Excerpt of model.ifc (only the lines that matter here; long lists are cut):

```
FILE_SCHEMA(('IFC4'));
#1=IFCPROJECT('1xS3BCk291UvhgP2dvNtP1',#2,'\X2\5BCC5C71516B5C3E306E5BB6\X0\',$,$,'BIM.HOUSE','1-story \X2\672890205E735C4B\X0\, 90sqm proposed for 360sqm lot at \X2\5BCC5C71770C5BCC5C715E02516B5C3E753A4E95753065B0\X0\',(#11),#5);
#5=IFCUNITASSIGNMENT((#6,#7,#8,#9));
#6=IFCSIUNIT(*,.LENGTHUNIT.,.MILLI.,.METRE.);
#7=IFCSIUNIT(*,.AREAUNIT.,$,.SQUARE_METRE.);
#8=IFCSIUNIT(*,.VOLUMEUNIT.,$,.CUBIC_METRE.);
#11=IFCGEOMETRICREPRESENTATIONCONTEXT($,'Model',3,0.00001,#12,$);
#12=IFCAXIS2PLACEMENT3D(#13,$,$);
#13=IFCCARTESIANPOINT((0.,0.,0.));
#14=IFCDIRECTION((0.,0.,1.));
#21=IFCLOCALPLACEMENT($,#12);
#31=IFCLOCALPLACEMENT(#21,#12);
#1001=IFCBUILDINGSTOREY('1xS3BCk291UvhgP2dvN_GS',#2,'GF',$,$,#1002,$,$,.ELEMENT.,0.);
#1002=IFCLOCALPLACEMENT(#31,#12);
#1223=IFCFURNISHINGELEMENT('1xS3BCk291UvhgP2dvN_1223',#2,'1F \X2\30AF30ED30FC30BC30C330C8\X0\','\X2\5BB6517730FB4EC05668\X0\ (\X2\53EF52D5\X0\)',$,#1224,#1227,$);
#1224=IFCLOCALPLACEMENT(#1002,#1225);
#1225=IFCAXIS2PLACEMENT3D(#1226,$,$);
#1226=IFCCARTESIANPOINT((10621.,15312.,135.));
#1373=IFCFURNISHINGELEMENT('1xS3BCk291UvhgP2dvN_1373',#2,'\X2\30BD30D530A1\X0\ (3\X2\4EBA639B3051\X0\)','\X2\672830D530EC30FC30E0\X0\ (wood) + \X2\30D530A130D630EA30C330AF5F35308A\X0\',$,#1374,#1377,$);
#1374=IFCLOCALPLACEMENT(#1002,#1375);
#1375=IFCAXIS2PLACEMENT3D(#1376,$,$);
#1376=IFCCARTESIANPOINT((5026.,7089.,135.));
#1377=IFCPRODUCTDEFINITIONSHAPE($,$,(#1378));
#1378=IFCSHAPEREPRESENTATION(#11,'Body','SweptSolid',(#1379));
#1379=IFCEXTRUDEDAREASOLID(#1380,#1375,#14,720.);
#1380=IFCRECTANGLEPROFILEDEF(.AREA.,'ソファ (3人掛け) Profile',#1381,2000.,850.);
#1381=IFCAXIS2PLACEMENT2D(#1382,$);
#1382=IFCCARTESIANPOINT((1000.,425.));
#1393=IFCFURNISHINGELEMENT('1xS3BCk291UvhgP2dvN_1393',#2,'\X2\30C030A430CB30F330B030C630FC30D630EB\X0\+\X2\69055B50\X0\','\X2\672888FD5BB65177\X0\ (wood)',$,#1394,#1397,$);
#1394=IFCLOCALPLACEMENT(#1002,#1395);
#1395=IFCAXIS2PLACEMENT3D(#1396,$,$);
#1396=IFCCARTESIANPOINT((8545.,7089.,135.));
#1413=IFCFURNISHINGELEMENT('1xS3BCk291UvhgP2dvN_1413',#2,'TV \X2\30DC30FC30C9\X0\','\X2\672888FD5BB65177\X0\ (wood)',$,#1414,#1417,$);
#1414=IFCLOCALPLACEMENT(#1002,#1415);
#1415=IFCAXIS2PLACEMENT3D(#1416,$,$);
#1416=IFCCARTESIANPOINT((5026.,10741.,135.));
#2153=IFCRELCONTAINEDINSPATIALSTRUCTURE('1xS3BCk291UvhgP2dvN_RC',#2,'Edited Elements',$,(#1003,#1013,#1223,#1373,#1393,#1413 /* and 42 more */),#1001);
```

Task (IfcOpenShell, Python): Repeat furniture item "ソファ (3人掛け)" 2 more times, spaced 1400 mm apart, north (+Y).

```python
import numpy as np
import ifcopenshell
import ifcopenshell.api.geometry
import ifcopenshell.api.root
import ifcopenshell.util.element
import ifcopenshell.util.placement
import ifcopenshell.util.unit

model = ifcopenshell.open("model.ifc")
unit_scale = ifcopenshell.util.unit.calculate_unit_scale(model)


def reuse_history(source, copy):
    """copy_class also copies each property set's owner history, people and application; keep the originals."""
    for rel in copy.IsDefinedBy:
        if rel.is_a("IfcRelDefinesByProperties") and (history := rel.RelatingPropertyDefinition.OwnerHistory):
            rel.RelatingPropertyDefinition.OwnerHistory = source.OwnerHistory
            ifcopenshell.util.element.remove_deep2(model, history)


source = model.by_guid("1xS3BCk291UvhgP2dvN_1373")
base = ifcopenshell.util.placement.get_local_placement(source.ObjectPlacement)
step = np.array([0.0, 1.0, 0.0]) * 1.4 / unit_scale

for i in range(1, 3):
    copy = ifcopenshell.api.root.copy_class(model, product=source)
    copy.Representation = ifcopenshell.util.element.copy_deep(
        model, source.Representation, exclude=["IfcGeometricRepresentationContext", "IfcRepresentationMap"]
    )
    reuse_history(source, copy)
    matrix = base.copy()
    matrix[:3, 3] += i * step
    print("added at", matrix[:3, 3].round(3) + 0.0)
    ifcopenshell.api.geometry.edit_object_placement(model, product=copy, matrix=matrix, is_si=False)

model.write("model_v2.ifc")
```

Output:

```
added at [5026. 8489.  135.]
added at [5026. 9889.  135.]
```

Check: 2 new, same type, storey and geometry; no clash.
